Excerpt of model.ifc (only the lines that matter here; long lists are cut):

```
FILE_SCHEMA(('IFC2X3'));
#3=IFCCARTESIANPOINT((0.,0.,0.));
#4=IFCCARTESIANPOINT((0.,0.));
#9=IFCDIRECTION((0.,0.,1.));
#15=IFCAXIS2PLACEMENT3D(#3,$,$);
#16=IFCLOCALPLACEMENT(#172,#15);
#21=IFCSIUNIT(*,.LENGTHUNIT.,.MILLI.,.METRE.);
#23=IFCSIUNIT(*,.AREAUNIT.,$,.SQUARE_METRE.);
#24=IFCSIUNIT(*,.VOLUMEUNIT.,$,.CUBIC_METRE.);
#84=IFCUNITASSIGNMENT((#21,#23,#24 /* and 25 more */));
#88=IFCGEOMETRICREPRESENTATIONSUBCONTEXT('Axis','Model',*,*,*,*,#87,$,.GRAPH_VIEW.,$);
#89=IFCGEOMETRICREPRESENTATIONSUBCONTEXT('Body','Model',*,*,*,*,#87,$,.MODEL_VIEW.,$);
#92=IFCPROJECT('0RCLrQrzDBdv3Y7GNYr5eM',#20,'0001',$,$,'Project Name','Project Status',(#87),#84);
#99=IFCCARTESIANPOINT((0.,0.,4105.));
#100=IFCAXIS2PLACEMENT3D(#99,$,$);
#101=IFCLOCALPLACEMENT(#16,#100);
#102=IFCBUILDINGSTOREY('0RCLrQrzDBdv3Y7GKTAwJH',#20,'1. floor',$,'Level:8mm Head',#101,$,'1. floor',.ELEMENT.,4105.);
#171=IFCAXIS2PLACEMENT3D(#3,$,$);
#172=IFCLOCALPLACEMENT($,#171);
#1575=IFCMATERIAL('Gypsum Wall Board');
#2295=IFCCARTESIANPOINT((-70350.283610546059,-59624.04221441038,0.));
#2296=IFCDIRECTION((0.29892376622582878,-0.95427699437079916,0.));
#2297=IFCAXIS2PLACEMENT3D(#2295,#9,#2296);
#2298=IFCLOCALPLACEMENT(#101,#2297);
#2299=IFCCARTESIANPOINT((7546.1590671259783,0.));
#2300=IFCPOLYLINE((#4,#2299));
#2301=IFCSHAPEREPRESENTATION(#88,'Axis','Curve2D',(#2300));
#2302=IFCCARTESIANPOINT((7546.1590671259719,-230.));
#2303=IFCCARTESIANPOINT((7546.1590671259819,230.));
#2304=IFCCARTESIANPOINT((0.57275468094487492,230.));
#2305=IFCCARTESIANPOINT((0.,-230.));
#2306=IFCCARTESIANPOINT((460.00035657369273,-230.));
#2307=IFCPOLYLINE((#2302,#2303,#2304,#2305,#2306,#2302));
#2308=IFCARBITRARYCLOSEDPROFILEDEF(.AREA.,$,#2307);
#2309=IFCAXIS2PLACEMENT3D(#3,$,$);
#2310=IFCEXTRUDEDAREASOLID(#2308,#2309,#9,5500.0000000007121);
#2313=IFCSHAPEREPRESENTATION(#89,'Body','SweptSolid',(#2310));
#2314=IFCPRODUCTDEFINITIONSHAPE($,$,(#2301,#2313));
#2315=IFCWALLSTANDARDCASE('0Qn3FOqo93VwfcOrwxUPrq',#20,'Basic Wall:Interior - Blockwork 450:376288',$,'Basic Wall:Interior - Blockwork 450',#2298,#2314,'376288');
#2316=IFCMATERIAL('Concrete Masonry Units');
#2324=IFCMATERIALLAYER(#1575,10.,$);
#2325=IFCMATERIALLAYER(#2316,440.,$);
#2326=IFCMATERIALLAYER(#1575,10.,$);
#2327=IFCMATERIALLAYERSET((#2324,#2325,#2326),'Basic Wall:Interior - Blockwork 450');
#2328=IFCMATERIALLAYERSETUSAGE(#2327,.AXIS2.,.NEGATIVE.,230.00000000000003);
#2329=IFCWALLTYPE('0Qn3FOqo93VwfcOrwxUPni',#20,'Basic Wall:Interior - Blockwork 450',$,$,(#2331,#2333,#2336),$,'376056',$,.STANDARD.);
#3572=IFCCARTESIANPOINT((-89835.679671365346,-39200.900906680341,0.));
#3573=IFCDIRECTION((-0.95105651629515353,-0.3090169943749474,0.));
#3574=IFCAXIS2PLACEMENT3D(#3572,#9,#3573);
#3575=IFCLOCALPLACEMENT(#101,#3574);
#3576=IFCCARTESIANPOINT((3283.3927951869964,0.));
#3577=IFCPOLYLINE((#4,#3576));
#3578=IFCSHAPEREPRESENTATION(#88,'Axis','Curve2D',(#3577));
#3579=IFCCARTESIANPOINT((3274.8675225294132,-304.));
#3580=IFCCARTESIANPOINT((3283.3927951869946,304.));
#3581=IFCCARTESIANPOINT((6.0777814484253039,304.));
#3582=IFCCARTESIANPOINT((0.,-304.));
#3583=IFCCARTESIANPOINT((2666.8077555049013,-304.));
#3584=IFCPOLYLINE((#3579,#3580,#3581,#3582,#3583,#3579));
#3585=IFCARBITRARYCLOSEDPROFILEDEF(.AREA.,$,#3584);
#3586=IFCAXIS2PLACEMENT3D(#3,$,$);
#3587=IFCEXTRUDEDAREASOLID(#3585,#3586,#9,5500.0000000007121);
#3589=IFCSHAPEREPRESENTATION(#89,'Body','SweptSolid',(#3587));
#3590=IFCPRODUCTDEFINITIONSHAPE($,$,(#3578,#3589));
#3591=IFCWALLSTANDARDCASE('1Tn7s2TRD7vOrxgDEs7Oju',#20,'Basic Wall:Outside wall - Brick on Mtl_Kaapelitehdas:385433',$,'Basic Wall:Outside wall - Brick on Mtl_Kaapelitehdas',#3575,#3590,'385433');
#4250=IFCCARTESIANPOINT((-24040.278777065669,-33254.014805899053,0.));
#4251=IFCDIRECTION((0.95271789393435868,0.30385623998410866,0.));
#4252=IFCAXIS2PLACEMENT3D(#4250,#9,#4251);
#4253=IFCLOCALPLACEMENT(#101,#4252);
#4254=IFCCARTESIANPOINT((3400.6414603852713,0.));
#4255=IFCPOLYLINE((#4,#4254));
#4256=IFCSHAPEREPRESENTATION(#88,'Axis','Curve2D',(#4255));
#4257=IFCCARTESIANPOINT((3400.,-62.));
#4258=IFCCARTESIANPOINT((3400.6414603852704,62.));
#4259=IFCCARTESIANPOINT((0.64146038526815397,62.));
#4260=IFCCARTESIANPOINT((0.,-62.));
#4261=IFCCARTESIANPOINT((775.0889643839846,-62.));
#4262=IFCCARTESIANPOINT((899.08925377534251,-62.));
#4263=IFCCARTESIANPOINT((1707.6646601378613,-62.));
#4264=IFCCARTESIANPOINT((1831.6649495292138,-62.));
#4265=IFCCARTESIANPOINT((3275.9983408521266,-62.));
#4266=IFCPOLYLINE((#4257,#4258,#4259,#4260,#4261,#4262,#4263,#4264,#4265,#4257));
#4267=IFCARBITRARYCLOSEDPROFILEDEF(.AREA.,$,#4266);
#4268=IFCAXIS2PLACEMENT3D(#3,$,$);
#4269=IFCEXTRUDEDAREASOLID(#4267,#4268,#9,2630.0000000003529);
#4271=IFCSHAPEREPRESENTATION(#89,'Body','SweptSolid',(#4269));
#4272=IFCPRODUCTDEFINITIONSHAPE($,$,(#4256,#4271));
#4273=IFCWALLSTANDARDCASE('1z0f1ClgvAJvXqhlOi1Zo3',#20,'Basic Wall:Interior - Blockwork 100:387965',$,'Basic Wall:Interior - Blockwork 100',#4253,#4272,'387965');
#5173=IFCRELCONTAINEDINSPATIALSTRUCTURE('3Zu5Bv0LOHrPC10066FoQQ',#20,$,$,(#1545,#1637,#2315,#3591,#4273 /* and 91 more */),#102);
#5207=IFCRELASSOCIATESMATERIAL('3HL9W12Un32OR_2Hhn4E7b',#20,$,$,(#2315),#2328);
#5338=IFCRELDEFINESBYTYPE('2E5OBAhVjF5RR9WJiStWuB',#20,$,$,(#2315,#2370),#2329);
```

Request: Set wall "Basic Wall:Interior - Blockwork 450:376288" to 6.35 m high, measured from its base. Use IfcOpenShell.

```python
import ifcopenshell
import ifcopenshell.geom
import ifcopenshell.util.representation
import ifcopenshell.util.shape

model = ifcopenshell.open("model.ifc")
settings = ifcopenshell.geom.settings()


def volume(element):
    """Net volume in cubic metres, openings subtracted."""
    shape = ifcopenshell.geom.create_shape(settings, element)
    return ifcopenshell.util.shape.get_volume(shape.geometry)


wall = model.by_guid("0Qn3FOqo93VwfcOrwxUPrq")
before = volume(wall)

body = ifcopenshell.util.representation.get_representation(wall, "Model", "Body")
solid = body.Items[0]
old_height = solid.Depth
solid.Depth = 6350.0
after = volume(wall)

print(f"height {old_height:g} -> {solid.Depth:g}, volume {before:.3f} -> {after:.3f} m3")

model.write("model_edited.ifc")
```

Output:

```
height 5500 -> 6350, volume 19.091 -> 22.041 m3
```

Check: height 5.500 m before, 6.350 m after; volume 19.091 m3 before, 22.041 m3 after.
